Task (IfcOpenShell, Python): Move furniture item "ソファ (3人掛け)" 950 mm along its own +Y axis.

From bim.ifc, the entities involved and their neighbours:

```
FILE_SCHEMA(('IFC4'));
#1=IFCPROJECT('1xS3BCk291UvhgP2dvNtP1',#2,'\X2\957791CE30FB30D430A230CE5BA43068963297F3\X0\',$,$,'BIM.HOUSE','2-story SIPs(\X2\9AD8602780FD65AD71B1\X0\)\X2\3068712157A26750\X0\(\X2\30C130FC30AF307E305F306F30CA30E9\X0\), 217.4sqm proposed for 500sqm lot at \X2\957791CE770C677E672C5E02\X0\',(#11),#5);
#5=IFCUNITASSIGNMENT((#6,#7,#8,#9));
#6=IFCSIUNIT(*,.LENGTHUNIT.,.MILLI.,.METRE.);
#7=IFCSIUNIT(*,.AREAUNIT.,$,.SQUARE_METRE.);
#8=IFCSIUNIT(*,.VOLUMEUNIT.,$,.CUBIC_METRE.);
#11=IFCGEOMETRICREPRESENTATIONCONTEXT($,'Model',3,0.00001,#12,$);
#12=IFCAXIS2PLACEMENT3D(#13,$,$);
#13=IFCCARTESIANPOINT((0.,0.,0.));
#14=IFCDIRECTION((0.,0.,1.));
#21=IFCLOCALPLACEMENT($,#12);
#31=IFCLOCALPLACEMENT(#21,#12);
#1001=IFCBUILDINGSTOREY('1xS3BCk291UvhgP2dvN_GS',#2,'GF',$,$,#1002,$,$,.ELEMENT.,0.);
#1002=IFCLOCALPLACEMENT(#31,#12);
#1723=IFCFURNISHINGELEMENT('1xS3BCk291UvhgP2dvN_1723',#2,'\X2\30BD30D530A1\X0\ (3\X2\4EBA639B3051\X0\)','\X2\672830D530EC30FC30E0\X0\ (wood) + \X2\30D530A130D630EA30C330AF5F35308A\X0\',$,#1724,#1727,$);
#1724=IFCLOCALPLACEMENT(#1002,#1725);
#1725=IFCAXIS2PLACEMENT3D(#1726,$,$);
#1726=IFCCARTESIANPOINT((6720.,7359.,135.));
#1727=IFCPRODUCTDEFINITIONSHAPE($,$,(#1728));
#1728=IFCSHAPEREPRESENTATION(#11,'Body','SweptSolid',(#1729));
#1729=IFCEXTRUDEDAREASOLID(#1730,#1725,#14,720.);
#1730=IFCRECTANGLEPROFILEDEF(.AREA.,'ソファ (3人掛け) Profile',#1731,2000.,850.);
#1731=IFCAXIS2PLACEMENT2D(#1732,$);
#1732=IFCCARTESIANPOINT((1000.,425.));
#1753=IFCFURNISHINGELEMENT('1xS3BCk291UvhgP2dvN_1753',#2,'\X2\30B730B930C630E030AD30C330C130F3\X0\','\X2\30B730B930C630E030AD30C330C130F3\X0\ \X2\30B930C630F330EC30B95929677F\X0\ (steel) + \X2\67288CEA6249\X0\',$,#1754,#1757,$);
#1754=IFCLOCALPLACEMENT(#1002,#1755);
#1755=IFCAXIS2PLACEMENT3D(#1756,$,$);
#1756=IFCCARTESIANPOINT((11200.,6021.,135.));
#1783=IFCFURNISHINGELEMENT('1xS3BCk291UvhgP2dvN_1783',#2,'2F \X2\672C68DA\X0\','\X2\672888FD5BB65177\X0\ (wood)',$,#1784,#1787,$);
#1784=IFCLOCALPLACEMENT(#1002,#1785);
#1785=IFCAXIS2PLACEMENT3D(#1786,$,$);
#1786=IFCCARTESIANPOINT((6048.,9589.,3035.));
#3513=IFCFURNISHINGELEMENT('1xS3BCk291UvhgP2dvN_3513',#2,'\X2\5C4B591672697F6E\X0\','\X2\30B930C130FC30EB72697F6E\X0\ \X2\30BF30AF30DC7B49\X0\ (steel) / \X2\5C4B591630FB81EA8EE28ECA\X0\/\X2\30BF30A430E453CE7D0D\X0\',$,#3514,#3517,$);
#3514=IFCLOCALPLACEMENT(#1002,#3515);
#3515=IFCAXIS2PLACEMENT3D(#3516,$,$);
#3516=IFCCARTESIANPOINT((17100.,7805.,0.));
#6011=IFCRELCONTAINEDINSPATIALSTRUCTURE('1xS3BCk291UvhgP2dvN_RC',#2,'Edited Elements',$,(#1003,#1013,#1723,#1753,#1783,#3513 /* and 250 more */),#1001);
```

```python
import ifcopenshell
import ifcopenshell.api.geometry
import ifcopenshell.util.placement
import ifcopenshell.util.unit

model = ifcopenshell.open("bim.ifc")
unit_scale = ifcopenshell.util.unit.calculate_unit_scale(model)

item = model.by_id(1723)
matrix = ifcopenshell.util.placement.get_local_placement(item.ObjectPlacement)
matrix[:3, 3] += matrix[:3, 1] * 0.95 / unit_scale
ifcopenshell.api.geometry.edit_object_placement(model, product=item, matrix=matrix, is_si=False)

print(ifcopenshell.util.placement.get_local_placement(item.ObjectPlacement).round(3) + 0.0)

model.write("bim_v2.ifc")
```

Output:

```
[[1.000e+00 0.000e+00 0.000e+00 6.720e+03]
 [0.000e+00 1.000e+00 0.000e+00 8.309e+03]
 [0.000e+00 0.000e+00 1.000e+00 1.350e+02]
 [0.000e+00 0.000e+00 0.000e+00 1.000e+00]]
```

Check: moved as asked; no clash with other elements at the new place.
